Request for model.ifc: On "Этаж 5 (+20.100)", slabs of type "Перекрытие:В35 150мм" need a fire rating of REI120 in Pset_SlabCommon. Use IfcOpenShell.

First a look at what the model holds.

```python
import ifcopenshell
import ifcopenshell.util.element

model = ifcopenshell.open("model.ifc")
print(model.schema)
storey = next(s for s in model.by_type("IfcBuildingStorey") if s.Name == "Этаж 5 (+20.100)")
slabs = [e for e in ifcopenshell.util.element.get_decomposition(storey) if e.is_a("IfcSlab")]
seen = {}
for e in slabs:
    element_type = ifcopenshell.util.element.get_type(e)
    key = (element_type.Name if element_type != e and element_type else None, ifcopenshell.util.element.get_pset(e, "Pset_SlabCommon", "FireRating"))
    seen[key] = seen.get(key, 0) + 1
for (name, value), count in sorted(seen.items(), key=str):
    print(count, "x", name, "|", value)
```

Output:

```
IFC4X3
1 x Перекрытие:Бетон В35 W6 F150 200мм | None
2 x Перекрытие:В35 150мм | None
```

```python
import ifcopenshell
import ifcopenshell.api.pset
import ifcopenshell.util.element

model = ifcopenshell.open("model.ifc")

storey = next(s for s in model.by_type("IfcBuildingStorey") if s.Name == "Этаж 5 (+20.100)")
slabs = [e for e in ifcopenshell.util.element.get_decomposition(storey) if e.is_a("IfcSlab")]

count = 0
for e in slabs:
    element_type = ifcopenshell.util.element.get_type(e)
    if element_type in (None, e) or element_type.Name != "Перекрытие:В35 150мм":
        continue
    # add_pset returns the element's existing set when there is one.
    pset = ifcopenshell.api.pset.add_pset(model, product=e, name="Pset_SlabCommon")
    ifcopenshell.api.pset.edit_pset(model, pset=pset, properties={"FireRating": "REI120"})
    count += 1

print(count, "slabs updated")

model.write("model_v2.ifc")
```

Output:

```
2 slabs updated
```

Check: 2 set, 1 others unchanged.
